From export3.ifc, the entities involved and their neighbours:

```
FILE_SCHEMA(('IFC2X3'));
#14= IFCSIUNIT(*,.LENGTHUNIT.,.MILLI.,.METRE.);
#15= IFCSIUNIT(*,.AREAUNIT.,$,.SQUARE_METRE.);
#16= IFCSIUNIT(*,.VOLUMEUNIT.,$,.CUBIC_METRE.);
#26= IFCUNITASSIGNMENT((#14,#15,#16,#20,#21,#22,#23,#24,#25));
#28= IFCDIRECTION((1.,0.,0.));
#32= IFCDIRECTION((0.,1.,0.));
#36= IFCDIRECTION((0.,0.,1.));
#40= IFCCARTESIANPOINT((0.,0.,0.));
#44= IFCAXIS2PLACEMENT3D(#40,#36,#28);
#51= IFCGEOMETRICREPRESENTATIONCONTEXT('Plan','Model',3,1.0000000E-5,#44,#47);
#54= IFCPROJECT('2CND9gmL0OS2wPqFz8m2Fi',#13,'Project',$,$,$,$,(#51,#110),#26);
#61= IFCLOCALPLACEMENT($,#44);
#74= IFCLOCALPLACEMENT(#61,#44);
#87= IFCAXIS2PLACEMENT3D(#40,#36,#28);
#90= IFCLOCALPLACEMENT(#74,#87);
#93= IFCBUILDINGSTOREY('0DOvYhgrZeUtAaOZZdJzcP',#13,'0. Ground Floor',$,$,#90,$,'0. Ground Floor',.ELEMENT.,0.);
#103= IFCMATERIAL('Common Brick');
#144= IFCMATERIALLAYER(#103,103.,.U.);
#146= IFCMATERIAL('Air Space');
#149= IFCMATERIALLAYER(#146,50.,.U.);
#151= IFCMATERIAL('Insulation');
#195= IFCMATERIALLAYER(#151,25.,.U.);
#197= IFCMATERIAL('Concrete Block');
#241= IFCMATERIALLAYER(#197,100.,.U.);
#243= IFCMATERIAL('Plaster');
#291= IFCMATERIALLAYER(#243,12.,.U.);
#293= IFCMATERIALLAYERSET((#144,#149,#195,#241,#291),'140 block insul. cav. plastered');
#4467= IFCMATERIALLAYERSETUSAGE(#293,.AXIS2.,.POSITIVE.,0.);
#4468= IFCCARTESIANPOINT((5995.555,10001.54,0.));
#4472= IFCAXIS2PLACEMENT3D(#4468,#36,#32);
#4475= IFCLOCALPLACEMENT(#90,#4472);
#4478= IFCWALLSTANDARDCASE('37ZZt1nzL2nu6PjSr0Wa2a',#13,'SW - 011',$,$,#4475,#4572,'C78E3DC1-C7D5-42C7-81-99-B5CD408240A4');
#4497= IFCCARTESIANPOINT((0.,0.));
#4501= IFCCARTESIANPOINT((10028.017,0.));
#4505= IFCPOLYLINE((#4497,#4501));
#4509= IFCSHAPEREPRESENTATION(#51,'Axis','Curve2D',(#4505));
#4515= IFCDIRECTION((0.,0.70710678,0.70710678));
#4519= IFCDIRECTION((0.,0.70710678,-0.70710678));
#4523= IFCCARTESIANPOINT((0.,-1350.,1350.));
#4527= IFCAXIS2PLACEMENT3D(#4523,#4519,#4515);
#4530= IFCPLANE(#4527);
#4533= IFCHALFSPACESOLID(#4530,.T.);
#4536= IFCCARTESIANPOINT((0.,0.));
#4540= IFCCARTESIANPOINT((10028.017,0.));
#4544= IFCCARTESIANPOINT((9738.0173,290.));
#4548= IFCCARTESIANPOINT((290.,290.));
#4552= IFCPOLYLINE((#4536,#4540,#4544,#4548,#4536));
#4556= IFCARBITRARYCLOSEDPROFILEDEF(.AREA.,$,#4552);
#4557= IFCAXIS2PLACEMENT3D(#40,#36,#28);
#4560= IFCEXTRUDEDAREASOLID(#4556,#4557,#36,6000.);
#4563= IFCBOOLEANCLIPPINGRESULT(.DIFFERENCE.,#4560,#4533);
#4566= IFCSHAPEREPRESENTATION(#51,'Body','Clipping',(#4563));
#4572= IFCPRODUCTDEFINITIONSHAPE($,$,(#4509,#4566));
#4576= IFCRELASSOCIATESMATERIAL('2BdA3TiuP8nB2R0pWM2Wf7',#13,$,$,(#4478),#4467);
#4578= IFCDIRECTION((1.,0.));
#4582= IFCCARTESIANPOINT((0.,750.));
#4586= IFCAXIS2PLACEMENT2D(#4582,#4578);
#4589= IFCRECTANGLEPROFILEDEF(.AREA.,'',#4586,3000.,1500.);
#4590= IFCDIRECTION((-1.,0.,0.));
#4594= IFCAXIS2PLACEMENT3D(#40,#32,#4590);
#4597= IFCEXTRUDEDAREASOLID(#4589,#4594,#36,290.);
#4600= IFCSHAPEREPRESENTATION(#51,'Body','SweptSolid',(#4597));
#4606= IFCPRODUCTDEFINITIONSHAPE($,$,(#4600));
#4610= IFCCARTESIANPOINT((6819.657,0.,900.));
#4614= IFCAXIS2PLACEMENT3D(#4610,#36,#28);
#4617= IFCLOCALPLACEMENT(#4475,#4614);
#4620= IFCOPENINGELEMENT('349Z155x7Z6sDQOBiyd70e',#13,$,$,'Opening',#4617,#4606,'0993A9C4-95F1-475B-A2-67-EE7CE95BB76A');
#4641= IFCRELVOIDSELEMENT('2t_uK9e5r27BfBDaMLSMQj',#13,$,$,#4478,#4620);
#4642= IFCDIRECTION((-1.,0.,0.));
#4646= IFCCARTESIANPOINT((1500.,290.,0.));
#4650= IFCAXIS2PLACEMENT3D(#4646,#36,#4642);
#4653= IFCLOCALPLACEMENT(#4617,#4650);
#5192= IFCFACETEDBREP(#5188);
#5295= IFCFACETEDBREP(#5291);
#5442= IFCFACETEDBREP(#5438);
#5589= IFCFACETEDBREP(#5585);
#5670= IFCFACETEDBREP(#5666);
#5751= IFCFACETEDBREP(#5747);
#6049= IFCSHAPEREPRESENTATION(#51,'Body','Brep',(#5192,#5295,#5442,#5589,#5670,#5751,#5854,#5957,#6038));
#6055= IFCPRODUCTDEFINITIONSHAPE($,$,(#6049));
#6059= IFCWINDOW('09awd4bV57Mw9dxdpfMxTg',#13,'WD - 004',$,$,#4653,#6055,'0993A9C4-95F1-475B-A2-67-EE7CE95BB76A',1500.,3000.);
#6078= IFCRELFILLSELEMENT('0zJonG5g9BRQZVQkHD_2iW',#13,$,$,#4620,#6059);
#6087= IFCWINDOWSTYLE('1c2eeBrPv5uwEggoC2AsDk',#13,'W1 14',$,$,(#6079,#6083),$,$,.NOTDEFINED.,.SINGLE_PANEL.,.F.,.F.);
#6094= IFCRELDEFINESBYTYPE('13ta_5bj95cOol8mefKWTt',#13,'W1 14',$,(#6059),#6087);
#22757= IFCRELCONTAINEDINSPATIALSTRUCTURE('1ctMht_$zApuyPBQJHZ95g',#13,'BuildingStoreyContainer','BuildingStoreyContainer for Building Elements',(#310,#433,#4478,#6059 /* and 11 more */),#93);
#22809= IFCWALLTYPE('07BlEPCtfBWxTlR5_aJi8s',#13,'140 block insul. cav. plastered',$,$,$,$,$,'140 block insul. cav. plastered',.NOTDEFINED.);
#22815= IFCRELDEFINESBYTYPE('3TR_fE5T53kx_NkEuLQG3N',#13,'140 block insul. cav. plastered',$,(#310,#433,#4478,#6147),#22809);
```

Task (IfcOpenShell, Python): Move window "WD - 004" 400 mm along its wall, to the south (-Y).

```python
import ifcopenshell
import ifcopenshell.api.geometry
import ifcopenshell.util.placement

model = ifcopenshell.open("export3.ifc")

window = model.by_guid("09awd4bV57Mw9dxdpfMxTg")
opening = window.FillsVoids[0].RelatingOpeningElement
wall = opening.VoidsElements[0].RelatingBuildingElement

wall_matrix = ifcopenshell.util.placement.get_local_placement(wall.ObjectPlacement)
shift = wall_matrix[:3, 0] * -400.0
before = ifcopenshell.util.placement.get_local_placement(window.ObjectPlacement)[:3, 3].copy()

# The window is placed relative to its opening, so it follows when the opening moves.
matrix = ifcopenshell.util.placement.get_local_placement(opening.ObjectPlacement)
matrix[:3, 3] += shift
ifcopenshell.api.geometry.edit_object_placement(
    model, product=opening, matrix=matrix, is_si=False, should_transform_children=True
)

after = ifcopenshell.util.placement.get_local_placement(window.ObjectPlacement)[:3, 3]
print("window moved by", (after - before).round(3) + 0.0)

model.write("export3_v2.ifc")
```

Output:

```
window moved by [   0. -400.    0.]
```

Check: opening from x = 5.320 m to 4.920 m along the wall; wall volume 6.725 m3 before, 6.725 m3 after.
